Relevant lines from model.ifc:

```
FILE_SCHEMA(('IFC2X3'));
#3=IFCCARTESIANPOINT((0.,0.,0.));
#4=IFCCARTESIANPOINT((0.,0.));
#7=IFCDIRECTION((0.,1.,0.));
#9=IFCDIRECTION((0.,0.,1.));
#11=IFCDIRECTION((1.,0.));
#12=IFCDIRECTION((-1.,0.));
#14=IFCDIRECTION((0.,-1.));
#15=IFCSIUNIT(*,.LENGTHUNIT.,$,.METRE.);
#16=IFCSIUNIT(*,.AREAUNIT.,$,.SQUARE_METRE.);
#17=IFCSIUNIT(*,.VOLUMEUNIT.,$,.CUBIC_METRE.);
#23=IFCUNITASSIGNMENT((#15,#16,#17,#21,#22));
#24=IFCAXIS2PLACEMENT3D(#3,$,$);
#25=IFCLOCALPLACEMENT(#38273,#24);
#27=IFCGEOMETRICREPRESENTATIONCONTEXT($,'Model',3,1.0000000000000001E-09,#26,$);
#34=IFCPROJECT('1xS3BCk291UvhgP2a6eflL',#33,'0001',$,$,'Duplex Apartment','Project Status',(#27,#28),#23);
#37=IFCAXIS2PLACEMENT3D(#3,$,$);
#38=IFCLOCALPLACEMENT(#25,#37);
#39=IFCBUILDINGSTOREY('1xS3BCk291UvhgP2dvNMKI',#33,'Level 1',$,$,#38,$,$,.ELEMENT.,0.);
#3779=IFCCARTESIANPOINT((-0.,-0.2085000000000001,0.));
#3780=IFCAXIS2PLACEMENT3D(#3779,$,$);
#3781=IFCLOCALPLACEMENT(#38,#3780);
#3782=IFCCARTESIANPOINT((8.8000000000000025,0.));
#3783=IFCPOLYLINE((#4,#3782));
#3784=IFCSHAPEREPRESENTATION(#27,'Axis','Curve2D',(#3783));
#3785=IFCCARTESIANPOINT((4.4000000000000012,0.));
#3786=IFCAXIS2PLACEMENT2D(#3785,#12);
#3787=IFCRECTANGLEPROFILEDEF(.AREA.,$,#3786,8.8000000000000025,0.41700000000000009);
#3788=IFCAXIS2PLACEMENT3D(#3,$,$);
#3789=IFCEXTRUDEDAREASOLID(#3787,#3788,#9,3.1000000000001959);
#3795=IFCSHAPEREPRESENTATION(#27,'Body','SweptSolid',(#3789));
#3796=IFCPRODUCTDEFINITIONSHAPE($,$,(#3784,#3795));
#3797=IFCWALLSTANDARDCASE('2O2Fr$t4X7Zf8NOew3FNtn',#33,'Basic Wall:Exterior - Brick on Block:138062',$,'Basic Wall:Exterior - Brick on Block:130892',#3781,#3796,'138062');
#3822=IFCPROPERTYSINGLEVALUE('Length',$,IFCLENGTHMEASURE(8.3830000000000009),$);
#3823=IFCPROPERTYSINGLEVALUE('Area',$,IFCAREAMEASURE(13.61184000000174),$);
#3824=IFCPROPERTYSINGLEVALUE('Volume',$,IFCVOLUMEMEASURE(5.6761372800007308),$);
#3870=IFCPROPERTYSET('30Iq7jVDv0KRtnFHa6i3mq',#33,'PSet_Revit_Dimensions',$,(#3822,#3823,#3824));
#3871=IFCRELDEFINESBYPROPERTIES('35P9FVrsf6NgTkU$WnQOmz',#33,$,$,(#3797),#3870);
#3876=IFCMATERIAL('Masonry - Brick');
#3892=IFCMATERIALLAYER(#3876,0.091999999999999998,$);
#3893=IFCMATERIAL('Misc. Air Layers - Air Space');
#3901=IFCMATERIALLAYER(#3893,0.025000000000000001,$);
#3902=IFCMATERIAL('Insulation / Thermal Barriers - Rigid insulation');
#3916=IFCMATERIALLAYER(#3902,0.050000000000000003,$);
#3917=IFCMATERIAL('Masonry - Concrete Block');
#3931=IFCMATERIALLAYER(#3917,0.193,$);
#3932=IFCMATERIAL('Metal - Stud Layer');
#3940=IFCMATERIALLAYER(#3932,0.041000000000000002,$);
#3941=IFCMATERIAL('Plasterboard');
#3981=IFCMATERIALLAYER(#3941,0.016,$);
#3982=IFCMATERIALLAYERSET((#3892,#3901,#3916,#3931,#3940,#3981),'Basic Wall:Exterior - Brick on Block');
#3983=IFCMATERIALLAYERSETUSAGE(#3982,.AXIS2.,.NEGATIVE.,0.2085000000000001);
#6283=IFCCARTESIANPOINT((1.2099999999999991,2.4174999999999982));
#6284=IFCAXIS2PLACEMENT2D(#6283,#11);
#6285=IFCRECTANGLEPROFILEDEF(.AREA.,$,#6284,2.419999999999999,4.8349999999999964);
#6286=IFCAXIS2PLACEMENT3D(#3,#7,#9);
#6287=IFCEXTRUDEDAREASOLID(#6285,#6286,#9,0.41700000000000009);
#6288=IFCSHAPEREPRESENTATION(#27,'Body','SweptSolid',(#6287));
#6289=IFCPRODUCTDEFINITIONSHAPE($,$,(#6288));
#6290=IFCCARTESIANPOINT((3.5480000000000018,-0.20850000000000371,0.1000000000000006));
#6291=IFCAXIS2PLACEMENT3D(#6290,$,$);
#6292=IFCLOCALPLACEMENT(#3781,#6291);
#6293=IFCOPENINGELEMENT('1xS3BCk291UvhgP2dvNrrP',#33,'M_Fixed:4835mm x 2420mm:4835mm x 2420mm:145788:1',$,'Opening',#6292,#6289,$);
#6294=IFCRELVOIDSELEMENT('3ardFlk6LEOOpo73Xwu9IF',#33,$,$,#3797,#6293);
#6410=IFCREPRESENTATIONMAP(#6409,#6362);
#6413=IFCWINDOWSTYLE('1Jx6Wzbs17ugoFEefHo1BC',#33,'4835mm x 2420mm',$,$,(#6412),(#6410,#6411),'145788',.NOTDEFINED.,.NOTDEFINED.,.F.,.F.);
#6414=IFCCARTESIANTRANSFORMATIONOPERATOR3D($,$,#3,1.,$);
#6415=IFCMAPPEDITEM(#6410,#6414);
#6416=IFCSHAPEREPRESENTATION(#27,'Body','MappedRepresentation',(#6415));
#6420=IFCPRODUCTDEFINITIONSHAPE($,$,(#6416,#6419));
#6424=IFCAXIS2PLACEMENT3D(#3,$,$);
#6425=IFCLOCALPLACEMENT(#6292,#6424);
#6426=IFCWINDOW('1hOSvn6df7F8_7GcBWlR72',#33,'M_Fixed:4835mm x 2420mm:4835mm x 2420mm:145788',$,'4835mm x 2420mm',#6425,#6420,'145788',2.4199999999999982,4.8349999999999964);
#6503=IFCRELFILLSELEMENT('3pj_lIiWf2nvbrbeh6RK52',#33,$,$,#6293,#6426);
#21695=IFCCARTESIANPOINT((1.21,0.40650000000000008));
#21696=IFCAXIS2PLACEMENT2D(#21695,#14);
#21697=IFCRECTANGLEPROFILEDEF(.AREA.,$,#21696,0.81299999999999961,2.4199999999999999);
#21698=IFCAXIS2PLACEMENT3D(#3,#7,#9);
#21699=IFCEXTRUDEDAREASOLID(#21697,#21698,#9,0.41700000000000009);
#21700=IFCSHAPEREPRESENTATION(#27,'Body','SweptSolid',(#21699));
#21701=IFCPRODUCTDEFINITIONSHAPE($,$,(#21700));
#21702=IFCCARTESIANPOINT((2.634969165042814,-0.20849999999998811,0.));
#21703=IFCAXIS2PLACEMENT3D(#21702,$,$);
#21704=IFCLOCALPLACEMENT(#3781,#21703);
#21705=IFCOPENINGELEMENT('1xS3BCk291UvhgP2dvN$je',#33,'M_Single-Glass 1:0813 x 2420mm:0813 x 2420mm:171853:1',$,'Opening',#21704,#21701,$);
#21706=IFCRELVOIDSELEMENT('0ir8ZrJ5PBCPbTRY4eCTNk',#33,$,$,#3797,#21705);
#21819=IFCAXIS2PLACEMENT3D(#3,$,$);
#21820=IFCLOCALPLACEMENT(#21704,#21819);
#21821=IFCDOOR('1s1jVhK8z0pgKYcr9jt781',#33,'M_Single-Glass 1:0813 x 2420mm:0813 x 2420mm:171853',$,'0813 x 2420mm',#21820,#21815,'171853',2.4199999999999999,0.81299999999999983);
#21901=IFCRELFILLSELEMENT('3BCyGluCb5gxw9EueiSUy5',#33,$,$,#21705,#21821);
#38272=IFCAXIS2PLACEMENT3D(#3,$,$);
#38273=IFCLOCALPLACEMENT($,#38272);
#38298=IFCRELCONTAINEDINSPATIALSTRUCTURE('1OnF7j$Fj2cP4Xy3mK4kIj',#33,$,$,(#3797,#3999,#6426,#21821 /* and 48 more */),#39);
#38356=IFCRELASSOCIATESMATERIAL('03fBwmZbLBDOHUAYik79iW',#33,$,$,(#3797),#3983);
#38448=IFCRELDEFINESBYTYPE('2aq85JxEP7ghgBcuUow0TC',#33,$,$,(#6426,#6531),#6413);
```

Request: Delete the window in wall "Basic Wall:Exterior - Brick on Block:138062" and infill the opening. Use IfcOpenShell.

```python
import ifcopenshell
import ifcopenshell.api.feature
import ifcopenshell.api.pset
import ifcopenshell.api.root
import ifcopenshell.geom
import ifcopenshell.util.element
import ifcopenshell.util.shape
import ifcopenshell.util.unit

model = ifcopenshell.open("model.ifc")
area_scale = ifcopenshell.util.unit.calculate_unit_scale(model, "AREAUNIT")
volume_scale = ifcopenshell.util.unit.calculate_unit_scale(model, "VOLUMEUNIT")
settings = ifcopenshell.geom.settings()


def volume(element):
    """Net volume in cubic metres, openings subtracted."""
    shape = ifcopenshell.geom.create_shape(settings, element)
    return ifcopenshell.util.shape.get_volume(shape.geometry)


window = model.by_guid("1hOSvn6df7F8_7GcBWlR72")
opening = window.FillsVoids[0].RelatingOpeningElement
wall = opening.VoidsElements[0].RelatingBuildingElement
before = volume(wall)

ifcopenshell.api.root.remove_product(model, product=window)
ifcopenshell.api.feature.remove_feature(model, feature=opening)

after = volume(wall)
thickness = 0.417  # wall thickness in metres

# Update the wall's stored quantities.
pset = model.by_id(ifcopenshell.util.element.get_pset(wall, "PSet_Revit_Dimensions", should_inherit=False)["id"])
ifcopenshell.api.pset.edit_pset(model, pset=pset, properties={
    "Area": model.create_entity("IfcAreaMeasure", after / thickness / area_scale),
    "Volume": model.create_entity("IfcVolumeMeasure", after / volume_scale),
})

print(f"wall volume {before:.3f} -> {after:.3f} m3")

model.write("model_rev.ifc")
```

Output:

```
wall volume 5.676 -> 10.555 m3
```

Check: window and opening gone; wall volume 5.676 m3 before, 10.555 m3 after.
